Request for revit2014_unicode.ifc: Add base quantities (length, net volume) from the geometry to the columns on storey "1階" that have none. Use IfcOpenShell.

First a look at what the model holds.

```python
import ifcopenshell
import ifcopenshell.util.element
import ifcopenshell.util.unit

model = ifcopenshell.open("revit2014_unicode.ifc")
print(model.schema)
for unit_type in ("LENGTHUNIT", "AREAUNIT", "VOLUMEUNIT"):
    print(unit_type, ifcopenshell.util.unit.calculate_unit_scale(model, unit_type))
storey = next(s for s in model.by_type("IfcBuildingStorey") if s.Name == "1階")
columns = [e for e in ifcopenshell.util.element.get_decomposition(storey) if e.is_a("IfcColumn")]
for e in sorted(columns, key=lambda e: e.id()):
    print(e.id(), e.is_a(), e.Name, list(ifcopenshell.util.element.get_psets(e, qtos_only=True)), sep=" | ")
```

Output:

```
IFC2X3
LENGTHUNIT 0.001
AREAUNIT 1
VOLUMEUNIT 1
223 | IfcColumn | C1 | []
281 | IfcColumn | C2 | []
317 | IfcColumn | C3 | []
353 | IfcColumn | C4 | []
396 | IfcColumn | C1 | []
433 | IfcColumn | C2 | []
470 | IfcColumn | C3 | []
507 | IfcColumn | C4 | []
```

```python
import ifcopenshell
import ifcopenshell.api.pset
import ifcopenshell.geom
import ifcopenshell.util.element
import ifcopenshell.util.shape
import ifcopenshell.util.unit

model = ifcopenshell.open("revit2014_unicode.ifc")
unit_scale = ifcopenshell.util.unit.calculate_unit_scale(model)
volume_scale = ifcopenshell.util.unit.calculate_unit_scale(model, "VOLUMEUNIT")
settings = ifcopenshell.geom.settings()

storey = next(s for s in model.by_type("IfcBuildingStorey") if s.Name == "1階")
columns = [e for e in ifcopenshell.util.element.get_decomposition(storey) if e.is_a("IfcColumn")]

for e in sorted(columns, key=lambda e: e.id()):
    if ifcopenshell.util.element.get_psets(e, qtos_only=True, should_inherit=False):
        continue
    # Geometry comes back in metres, in the element's own axes.
    shape = ifcopenshell.geom.create_shape(settings, e)
    values = {
        "Length": ifcopenshell.util.shape.get_z(shape.geometry) / unit_scale,
        "NetVolume": ifcopenshell.util.shape.get_volume(shape.geometry) / volume_scale,
    }
    qto = ifcopenshell.api.pset.add_qto(model, product=e, name="BaseQuantities")
    ifcopenshell.api.pset.edit_qto(model, qto=qto, properties=values)
    print(e.id(), {k: round(v, 3) for k, v in values.items()})

model.write("revit2014_unicode-out.ifc")
```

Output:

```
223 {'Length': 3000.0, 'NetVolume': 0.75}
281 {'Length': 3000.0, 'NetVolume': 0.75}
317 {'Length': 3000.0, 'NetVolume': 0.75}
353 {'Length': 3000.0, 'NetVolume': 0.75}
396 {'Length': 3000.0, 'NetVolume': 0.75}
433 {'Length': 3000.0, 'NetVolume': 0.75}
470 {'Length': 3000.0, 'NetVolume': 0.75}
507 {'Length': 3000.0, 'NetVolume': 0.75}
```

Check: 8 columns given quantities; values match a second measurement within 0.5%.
